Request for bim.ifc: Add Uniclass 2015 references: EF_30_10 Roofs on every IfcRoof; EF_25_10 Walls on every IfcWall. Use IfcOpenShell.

First a look at what the model holds.

```python
import ifcopenshell

model = ifcopenshell.open("bim.ifc")
print(model.schema)
print("classifications:", [c.Name for c in model.by_type("IfcClassification")])
for ifc_class in ("IfcDoor", "IfcRoof", "IfcStair", "IfcWall", "IfcWindow"):
    print(ifc_class, len(model.by_type(ifc_class)))
```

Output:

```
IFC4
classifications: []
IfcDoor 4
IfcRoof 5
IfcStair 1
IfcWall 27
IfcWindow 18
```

```python
import ifcopenshell
import ifcopenshell.api.classification

model = ifcopenshell.open("bim.ifc")

system = ifcopenshell.api.classification.add_classification(model, classification="Uniclass 2015")

codes = {
    "IfcRoof": ("EF_30_10", "Roofs"),
    "IfcWall": ("EF_25_10", "Walls"),
}
for ifc_class, (code, name) in codes.items():
    products = model.by_type(ifc_class)
    ifcopenshell.api.classification.add_reference(
        model, products=products, classification=system, identification=code, name=name
    )
    print(code, len(products))

model.write("bim_rev.ifc")
```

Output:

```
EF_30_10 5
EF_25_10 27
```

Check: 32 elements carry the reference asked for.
